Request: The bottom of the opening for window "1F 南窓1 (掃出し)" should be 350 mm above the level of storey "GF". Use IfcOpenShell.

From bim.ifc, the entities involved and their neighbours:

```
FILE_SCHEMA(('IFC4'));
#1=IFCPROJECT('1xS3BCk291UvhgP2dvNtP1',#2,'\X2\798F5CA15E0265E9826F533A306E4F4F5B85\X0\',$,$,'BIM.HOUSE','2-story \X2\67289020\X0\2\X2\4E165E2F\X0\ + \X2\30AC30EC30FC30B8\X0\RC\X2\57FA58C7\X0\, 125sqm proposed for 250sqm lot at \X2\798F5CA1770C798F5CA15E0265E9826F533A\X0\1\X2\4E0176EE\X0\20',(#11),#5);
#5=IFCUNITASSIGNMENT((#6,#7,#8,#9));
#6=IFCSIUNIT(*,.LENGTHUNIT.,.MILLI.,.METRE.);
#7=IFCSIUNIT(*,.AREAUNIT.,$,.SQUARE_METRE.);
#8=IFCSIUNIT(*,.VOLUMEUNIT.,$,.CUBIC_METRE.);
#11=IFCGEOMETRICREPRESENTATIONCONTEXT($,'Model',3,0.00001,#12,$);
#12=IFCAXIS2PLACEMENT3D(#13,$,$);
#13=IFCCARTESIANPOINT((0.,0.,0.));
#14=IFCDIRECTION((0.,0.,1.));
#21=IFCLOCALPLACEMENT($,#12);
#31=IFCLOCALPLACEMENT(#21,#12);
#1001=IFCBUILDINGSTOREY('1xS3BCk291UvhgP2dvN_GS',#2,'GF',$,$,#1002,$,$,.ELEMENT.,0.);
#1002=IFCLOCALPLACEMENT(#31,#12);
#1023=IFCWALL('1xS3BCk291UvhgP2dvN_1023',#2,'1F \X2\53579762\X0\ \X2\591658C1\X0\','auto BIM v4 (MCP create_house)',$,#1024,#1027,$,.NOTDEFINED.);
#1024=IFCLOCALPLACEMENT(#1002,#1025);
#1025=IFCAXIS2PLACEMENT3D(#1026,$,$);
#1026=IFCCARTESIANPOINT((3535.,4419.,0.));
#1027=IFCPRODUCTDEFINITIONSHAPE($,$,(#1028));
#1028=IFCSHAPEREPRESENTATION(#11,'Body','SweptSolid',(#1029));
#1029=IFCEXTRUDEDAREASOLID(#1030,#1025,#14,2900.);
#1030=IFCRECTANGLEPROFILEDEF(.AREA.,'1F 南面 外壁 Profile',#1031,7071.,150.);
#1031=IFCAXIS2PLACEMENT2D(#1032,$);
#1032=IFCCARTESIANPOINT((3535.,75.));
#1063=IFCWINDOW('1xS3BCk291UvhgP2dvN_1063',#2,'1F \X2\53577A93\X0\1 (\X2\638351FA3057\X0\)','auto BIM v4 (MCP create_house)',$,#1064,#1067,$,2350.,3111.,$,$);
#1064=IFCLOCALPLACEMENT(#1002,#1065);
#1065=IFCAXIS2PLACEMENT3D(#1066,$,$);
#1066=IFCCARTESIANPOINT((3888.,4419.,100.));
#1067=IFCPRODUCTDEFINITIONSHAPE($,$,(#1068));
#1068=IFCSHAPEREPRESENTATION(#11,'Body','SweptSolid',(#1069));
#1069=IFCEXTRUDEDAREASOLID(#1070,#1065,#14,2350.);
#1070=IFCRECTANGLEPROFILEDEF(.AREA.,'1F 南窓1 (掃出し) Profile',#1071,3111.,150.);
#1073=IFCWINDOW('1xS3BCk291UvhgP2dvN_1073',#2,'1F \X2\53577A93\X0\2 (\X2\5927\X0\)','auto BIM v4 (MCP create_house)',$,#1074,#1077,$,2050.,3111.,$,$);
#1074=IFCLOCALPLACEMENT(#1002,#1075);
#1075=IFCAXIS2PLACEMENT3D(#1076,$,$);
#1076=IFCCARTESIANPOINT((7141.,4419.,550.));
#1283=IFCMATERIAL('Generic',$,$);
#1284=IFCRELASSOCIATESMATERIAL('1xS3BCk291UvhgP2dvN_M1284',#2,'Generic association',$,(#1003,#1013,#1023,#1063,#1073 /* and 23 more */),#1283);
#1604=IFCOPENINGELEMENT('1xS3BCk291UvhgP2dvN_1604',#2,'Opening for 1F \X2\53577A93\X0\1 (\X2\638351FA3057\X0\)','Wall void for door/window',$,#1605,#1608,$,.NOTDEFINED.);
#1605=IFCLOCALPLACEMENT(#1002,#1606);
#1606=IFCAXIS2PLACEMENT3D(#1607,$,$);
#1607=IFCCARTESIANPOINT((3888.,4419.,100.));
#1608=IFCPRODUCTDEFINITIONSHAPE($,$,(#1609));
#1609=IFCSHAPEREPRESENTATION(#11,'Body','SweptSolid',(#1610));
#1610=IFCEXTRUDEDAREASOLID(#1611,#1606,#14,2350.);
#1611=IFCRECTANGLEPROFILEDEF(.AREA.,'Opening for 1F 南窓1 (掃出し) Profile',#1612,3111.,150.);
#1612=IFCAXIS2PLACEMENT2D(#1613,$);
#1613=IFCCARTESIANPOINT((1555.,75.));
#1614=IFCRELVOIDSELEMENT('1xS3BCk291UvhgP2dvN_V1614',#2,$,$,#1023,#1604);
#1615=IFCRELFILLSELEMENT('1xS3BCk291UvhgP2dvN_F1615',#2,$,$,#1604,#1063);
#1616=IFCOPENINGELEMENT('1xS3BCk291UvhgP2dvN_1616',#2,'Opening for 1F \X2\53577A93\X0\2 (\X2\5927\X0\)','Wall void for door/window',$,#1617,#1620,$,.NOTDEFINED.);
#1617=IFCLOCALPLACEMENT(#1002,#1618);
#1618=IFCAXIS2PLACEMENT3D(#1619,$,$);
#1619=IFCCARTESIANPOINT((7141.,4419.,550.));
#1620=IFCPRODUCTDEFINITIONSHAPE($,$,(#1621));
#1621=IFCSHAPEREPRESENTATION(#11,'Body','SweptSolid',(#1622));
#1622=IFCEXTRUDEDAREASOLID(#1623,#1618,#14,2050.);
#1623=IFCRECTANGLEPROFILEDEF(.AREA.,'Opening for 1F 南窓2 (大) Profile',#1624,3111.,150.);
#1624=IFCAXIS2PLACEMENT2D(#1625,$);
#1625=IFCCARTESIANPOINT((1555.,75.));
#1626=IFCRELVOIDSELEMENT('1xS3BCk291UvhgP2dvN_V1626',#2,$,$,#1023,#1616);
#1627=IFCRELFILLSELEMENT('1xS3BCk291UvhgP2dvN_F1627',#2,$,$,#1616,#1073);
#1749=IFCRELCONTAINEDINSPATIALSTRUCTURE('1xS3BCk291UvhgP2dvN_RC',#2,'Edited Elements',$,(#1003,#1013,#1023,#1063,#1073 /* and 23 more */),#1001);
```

```python
import numpy as np
import ifcopenshell
import ifcopenshell.api.geometry
import ifcopenshell.geom
import ifcopenshell.util.element
import ifcopenshell.util.placement
import ifcopenshell.util.shape
import ifcopenshell.util.unit

model = ifcopenshell.open("bim.ifc")
unit_scale = ifcopenshell.util.unit.calculate_unit_scale(model)

window = model.by_id(1063)
opening = window.FillsVoids[0].RelatingOpeningElement
storey = ifcopenshell.util.element.get_container(window, ifc_class="IfcBuildingStorey")
level = ifcopenshell.util.placement.get_local_placement(storey.ObjectPlacement)[2, 3]

# The opening's origin need not be at the sill, so measure its lowest point.
shape = ifcopenshell.geom.create_shape(ifcopenshell.geom.settings(), opening)
bottom = ifcopenshell.util.shape.get_shape_bottom_elevation(shape, shape.geometry) / unit_scale
dz = level + 350.0 - bottom

shift = np.array([0.0, 0.0, dz])
# The window is not placed relative to its opening, so move both.
for product in (opening, window):
    matrix = ifcopenshell.util.placement.get_local_placement(product.ObjectPlacement)
    matrix[:3, 3] += shift
    ifcopenshell.api.geometry.edit_object_placement(model, product=product, matrix=matrix, is_si=False)

print(f"moved by {dz * unit_scale:+.3f} m")

model.write("bim_updated.ifc")
```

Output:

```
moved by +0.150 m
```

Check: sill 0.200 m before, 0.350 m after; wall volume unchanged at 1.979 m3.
